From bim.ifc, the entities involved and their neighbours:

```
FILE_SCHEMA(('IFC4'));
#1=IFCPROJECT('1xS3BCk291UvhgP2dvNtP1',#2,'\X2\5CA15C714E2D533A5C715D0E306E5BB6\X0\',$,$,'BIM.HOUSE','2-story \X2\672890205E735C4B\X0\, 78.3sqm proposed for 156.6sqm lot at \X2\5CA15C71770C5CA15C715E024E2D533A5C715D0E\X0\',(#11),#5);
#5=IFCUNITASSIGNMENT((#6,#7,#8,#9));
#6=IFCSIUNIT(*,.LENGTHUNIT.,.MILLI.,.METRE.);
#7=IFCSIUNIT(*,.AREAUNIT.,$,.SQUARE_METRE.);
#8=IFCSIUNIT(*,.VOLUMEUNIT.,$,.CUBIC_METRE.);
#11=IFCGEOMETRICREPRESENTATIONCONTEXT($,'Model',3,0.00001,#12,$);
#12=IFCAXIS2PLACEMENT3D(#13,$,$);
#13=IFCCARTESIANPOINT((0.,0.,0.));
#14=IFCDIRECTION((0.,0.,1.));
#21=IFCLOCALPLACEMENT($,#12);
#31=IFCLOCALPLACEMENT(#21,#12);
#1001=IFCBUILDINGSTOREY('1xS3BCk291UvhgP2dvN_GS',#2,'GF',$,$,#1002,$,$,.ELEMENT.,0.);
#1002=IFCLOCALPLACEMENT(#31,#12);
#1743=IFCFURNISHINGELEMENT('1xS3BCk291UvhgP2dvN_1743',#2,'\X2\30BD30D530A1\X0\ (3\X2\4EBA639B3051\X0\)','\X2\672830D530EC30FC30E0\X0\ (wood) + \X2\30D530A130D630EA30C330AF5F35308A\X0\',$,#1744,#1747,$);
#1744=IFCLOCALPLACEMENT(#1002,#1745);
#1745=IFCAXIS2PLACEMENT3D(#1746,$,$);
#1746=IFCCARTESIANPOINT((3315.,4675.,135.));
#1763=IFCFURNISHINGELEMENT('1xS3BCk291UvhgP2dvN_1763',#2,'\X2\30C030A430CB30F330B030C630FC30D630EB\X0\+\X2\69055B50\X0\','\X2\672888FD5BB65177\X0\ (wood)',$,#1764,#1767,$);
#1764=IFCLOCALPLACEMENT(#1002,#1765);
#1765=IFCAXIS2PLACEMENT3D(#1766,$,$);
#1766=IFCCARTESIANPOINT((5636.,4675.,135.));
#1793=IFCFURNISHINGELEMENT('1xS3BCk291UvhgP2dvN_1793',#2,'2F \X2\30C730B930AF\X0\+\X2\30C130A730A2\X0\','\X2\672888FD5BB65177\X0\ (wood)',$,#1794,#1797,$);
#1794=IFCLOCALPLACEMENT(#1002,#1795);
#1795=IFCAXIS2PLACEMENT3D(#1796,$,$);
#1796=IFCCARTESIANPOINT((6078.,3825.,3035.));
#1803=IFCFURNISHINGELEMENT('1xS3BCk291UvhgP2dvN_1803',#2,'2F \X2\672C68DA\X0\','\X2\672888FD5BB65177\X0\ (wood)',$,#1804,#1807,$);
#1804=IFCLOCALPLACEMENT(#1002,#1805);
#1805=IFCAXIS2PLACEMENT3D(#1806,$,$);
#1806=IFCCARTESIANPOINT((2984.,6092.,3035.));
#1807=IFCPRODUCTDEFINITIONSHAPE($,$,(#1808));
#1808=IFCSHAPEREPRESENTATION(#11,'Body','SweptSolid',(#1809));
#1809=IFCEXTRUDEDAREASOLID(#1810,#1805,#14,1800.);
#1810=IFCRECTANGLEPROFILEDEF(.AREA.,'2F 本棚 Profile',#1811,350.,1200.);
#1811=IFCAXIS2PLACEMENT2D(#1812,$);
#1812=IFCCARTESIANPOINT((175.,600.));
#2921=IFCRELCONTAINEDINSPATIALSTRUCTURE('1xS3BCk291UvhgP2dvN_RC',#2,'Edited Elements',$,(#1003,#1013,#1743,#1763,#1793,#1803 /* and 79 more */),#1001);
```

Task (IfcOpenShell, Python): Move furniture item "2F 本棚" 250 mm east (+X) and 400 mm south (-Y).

```python
import ifcopenshell
import ifcopenshell.api.geometry
import ifcopenshell.util.placement
import ifcopenshell.util.unit

model = ifcopenshell.open("bim.ifc")
unit_scale = ifcopenshell.util.unit.calculate_unit_scale(model)

item = model.by_guid("1xS3BCk291UvhgP2dvN_1803")
matrix = ifcopenshell.util.placement.get_local_placement(item.ObjectPlacement)
matrix[0, 3] += 0.25 / unit_scale
matrix[1, 3] -= 0.4 / unit_scale
ifcopenshell.api.geometry.edit_object_placement(model, product=item, matrix=matrix, is_si=False)

print(ifcopenshell.util.placement.get_local_placement(item.ObjectPlacement).round(3) + 0.0)

model.write("bim-out.ifc")
```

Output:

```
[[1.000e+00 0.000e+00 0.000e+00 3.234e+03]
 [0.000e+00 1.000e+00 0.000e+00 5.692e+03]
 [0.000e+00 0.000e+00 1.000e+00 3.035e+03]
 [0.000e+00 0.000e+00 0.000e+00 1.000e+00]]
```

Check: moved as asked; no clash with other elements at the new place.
